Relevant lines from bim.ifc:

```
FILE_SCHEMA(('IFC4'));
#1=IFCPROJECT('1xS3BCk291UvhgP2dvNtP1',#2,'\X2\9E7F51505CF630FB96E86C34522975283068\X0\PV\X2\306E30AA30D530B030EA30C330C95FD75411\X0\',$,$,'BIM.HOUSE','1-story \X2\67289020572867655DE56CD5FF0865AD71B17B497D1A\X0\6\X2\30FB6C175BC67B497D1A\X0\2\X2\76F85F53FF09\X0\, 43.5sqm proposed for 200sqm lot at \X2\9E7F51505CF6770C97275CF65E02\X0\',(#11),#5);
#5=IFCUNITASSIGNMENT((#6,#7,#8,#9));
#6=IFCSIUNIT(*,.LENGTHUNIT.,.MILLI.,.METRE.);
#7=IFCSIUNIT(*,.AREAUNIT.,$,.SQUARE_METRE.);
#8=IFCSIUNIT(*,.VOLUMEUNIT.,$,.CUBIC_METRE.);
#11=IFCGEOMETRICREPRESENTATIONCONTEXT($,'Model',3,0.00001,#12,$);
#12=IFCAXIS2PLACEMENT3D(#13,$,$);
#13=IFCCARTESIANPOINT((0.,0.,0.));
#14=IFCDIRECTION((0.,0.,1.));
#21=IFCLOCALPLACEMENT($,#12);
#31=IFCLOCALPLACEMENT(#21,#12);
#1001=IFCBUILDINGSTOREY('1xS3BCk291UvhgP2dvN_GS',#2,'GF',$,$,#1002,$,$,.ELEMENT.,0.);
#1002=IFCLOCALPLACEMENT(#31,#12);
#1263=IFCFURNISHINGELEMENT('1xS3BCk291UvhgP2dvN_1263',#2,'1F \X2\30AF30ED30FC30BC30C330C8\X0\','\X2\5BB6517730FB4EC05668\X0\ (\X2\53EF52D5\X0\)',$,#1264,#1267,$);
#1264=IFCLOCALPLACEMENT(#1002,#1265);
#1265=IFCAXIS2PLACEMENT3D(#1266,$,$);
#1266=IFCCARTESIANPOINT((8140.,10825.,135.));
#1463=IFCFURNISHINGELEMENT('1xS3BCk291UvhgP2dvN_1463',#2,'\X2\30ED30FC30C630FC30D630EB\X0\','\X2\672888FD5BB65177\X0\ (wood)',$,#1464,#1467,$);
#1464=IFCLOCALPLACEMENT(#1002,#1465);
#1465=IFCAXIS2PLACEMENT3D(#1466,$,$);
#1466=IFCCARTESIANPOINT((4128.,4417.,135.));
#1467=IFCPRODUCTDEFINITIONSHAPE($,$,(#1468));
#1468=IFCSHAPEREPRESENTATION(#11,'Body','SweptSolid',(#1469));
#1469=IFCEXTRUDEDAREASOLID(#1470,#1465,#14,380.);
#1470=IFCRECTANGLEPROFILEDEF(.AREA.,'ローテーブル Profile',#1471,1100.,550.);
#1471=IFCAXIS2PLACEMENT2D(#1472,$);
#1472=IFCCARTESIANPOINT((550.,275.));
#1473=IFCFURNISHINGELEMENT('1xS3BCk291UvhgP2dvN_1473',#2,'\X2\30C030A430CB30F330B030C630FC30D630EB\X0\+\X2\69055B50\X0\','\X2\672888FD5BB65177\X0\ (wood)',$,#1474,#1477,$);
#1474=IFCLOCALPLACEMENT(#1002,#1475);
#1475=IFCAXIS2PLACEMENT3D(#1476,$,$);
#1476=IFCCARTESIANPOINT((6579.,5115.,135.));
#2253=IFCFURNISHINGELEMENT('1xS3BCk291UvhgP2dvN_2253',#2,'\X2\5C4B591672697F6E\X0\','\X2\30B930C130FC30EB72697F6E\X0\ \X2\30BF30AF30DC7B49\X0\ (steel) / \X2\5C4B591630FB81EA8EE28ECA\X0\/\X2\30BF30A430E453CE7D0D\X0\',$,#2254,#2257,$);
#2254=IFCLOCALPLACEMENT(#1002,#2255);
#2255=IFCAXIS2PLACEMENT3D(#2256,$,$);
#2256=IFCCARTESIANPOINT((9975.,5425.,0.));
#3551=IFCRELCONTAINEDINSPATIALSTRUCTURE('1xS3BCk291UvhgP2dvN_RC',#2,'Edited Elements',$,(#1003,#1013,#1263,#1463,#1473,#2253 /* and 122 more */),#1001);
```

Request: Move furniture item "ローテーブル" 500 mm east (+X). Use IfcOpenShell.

```python
import ifcopenshell
import ifcopenshell.api.geometry
import ifcopenshell.util.placement
import ifcopenshell.util.unit

model = ifcopenshell.open("bim.ifc")
unit_scale = ifcopenshell.util.unit.calculate_unit_scale(model)

item = model.by_guid("1xS3BCk291UvhgP2dvN_1463")
matrix = ifcopenshell.util.placement.get_local_placement(item.ObjectPlacement)
matrix[0, 3] += 0.5 / unit_scale
ifcopenshell.api.geometry.edit_object_placement(model, product=item, matrix=matrix, is_si=False)

print(ifcopenshell.util.placement.get_local_placement(item.ObjectPlacement).round(3) + 0.0)

model.write("bim_edited.ifc")
```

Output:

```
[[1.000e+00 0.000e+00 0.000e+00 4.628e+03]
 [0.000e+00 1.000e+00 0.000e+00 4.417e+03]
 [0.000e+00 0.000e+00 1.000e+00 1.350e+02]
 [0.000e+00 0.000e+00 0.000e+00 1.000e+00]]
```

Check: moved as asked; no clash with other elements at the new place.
